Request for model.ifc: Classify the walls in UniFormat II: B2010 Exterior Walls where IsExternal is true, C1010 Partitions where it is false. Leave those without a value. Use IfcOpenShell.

First a look at what the model holds.

```python
import ifcopenshell
import ifcopenshell.util.element

model = ifcopenshell.open("model.ifc")
print(model.schema)
print("classifications:", [c.Name for c in model.by_type("IfcClassification")])
values = [ifcopenshell.util.element.get_pset(e, "Pset_WallCommon", "IsExternal") for e in model.by_type("IfcWall")]
for value in (True, False, None):
    print("IsExternal", value, values.count(value))
```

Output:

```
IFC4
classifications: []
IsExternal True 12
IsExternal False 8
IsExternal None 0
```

```python
import ifcopenshell
import ifcopenshell.api.classification
import ifcopenshell.util.element

model = ifcopenshell.open("model.ifc")

system = ifcopenshell.api.classification.add_classification(model, classification="UniFormat II")

walls = model.by_type("IfcWall")
external = {e: ifcopenshell.util.element.get_pset(e, "Pset_WallCommon", "IsExternal") for e in walls}
for flag, code, name in ((True, "B2010", "Exterior Walls"), (False, "C1010", "Partitions")):
    products = [e for e in walls if external[e] is flag]
    ifcopenshell.api.classification.add_reference(
        model, products=products, classification=system, identification=code, name=name
    )
    print(code, len(products))

model.write("model_v2.ifc")
```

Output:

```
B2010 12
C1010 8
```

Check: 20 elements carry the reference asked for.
